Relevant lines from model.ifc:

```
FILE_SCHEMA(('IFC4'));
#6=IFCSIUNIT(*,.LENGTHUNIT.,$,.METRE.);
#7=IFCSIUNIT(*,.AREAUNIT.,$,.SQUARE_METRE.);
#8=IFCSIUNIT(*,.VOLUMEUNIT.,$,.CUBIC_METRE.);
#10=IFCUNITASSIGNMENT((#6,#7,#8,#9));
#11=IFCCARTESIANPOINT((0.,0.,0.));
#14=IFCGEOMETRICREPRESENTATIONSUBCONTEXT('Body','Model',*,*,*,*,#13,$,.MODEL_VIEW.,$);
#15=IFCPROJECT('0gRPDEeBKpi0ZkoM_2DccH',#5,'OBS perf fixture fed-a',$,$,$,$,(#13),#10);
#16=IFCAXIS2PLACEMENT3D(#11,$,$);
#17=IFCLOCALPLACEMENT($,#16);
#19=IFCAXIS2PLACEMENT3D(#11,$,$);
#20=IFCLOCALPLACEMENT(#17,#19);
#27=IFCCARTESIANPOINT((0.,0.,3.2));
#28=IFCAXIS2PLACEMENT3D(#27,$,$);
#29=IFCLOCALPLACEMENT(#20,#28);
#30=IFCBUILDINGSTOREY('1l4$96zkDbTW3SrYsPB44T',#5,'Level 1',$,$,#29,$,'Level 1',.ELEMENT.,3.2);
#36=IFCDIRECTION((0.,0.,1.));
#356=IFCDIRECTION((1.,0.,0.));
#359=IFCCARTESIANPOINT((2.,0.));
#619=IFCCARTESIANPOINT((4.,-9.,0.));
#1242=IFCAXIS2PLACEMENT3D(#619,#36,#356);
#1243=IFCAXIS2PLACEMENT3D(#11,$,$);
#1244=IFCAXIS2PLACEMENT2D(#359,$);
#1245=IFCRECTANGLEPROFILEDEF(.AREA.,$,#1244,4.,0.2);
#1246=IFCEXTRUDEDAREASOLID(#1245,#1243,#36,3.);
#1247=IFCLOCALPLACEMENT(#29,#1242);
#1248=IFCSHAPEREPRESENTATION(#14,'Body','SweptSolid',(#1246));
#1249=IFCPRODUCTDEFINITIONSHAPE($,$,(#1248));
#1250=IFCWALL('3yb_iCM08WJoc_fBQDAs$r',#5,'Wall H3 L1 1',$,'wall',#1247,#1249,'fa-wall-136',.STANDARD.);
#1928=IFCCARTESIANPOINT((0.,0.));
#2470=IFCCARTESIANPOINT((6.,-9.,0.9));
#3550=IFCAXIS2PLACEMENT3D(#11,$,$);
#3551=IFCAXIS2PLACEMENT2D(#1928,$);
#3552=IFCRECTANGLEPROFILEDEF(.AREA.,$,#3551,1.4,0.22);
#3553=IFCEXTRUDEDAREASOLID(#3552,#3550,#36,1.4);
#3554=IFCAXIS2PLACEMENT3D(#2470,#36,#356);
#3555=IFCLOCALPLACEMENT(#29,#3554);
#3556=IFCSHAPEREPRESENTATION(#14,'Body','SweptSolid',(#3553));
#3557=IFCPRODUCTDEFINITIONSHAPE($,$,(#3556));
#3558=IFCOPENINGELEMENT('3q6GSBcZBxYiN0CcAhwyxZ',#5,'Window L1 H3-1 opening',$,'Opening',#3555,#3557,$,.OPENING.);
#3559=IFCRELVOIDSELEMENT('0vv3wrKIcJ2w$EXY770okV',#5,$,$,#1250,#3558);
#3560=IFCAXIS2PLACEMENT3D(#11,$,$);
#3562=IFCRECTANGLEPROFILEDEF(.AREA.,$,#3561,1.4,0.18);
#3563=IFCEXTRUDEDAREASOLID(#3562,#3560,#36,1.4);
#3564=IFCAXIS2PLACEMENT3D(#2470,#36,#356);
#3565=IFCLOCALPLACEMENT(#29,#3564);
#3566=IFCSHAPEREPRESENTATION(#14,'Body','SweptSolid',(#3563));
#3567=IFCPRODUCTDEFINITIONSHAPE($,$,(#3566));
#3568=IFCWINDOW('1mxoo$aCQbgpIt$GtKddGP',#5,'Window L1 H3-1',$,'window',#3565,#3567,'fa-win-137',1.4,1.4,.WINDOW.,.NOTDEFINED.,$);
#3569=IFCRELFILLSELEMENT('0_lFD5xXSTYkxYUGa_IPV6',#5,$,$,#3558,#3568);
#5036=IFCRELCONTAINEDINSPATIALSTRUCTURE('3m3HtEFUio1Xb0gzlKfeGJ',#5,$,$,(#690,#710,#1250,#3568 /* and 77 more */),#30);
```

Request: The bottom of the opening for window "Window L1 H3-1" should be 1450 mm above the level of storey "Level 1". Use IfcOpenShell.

```python
import numpy as np
import ifcopenshell
import ifcopenshell.api.geometry
import ifcopenshell.geom
import ifcopenshell.util.element
import ifcopenshell.util.placement
import ifcopenshell.util.shape
import ifcopenshell.util.unit

model = ifcopenshell.open("model.ifc")
unit_scale = ifcopenshell.util.unit.calculate_unit_scale(model)

window = model.by_id(3568)
opening = window.FillsVoids[0].RelatingOpeningElement
storey = ifcopenshell.util.element.get_container(window, ifc_class="IfcBuildingStorey")
level = ifcopenshell.util.placement.get_local_placement(storey.ObjectPlacement)[2, 3]

# The opening's origin need not be at the sill, so measure its lowest point.
shape = ifcopenshell.geom.create_shape(ifcopenshell.geom.settings(), opening)
bottom = ifcopenshell.util.shape.get_shape_bottom_elevation(shape, shape.geometry) / unit_scale
dz = level + 1.45 - bottom

shift = np.array([0.0, 0.0, dz])
# The window is not placed relative to its opening, so move both.
for product in (opening, window):
    matrix = ifcopenshell.util.placement.get_local_placement(product.ObjectPlacement)
    matrix[:3, 3] += shift
    ifcopenshell.api.geometry.edit_object_placement(model, product=product, matrix=matrix, is_si=False)

print(f"moved by {dz * unit_scale:+.3f} m")

model.write("model_rev.ifc")
```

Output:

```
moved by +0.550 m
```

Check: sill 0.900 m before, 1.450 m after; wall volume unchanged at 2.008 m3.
